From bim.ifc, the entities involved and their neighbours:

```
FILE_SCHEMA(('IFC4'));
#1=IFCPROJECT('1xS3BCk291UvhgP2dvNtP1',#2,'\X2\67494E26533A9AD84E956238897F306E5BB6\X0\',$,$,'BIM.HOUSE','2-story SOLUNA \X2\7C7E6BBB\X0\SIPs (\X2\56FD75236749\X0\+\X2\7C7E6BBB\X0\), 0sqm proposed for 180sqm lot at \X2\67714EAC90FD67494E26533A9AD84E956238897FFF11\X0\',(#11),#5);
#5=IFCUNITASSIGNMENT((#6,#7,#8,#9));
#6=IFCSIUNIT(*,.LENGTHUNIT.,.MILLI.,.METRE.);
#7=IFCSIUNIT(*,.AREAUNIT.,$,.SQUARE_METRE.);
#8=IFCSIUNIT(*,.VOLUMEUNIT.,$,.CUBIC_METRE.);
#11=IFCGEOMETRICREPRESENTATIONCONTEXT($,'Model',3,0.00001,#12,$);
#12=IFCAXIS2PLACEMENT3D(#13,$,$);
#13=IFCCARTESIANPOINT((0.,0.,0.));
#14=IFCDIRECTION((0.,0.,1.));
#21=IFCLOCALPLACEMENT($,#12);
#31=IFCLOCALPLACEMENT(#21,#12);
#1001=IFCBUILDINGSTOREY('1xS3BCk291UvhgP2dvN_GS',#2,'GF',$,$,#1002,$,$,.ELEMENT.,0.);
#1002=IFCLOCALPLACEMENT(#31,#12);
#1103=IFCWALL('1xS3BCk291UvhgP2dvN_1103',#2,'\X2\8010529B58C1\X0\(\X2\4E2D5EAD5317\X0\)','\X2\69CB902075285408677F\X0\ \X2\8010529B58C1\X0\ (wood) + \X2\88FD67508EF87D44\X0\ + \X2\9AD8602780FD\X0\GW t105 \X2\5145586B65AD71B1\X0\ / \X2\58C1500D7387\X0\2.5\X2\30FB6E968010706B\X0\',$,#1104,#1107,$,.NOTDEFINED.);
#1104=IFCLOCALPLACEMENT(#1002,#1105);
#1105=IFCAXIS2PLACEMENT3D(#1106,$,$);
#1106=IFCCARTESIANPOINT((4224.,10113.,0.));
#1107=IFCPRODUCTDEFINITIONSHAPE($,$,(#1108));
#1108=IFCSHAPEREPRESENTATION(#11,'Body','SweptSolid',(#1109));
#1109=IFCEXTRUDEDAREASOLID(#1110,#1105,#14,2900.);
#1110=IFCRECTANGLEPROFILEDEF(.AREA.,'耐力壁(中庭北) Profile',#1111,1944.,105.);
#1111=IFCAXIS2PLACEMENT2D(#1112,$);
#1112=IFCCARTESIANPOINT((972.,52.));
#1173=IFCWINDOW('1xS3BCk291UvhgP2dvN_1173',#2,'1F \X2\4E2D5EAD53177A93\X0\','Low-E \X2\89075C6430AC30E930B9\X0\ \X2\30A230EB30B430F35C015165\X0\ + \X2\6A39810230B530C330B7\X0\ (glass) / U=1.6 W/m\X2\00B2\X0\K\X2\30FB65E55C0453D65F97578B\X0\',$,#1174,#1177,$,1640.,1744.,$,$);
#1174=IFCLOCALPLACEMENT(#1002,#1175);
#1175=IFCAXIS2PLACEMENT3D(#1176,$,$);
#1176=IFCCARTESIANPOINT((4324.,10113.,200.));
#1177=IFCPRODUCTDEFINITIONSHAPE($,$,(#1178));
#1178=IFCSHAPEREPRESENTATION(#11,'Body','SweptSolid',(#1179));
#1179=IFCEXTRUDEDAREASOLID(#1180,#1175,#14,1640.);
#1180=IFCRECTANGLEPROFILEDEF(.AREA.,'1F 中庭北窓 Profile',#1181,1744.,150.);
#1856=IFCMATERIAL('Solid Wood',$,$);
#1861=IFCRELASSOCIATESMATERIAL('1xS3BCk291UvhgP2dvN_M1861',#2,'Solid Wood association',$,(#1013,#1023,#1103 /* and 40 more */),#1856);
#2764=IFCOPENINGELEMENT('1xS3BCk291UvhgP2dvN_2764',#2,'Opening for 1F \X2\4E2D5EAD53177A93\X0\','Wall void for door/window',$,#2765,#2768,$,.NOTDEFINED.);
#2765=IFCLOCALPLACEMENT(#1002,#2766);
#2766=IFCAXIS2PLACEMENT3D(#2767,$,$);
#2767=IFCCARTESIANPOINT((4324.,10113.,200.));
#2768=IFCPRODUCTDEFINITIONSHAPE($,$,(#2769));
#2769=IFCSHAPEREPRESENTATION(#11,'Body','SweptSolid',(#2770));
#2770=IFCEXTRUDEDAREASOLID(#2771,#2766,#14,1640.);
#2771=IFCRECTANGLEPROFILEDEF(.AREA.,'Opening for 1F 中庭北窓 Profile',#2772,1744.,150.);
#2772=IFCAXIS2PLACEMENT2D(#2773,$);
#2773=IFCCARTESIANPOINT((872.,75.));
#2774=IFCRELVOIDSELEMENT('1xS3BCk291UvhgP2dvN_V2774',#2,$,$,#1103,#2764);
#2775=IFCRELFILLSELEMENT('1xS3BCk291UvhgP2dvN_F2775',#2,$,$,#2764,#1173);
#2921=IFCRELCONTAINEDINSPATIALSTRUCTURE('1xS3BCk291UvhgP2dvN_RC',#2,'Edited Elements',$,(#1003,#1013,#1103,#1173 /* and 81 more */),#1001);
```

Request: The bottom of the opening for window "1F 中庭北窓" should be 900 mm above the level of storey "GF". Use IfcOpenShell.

```python
import numpy as np
import ifcopenshell
import ifcopenshell.api.geometry
import ifcopenshell.geom
import ifcopenshell.util.element
import ifcopenshell.util.placement
import ifcopenshell.util.shape
import ifcopenshell.util.unit

model = ifcopenshell.open("bim.ifc")
unit_scale = ifcopenshell.util.unit.calculate_unit_scale(model)

window = model.by_id(1173)
opening = window.FillsVoids[0].RelatingOpeningElement
storey = ifcopenshell.util.element.get_container(window, ifc_class="IfcBuildingStorey")
level = ifcopenshell.util.placement.get_local_placement(storey.ObjectPlacement)[2, 3]

# The opening's origin need not be at the sill, so measure its lowest point.
shape = ifcopenshell.geom.create_shape(ifcopenshell.geom.settings(), opening)
bottom = ifcopenshell.util.shape.get_shape_bottom_elevation(shape, shape.geometry) / unit_scale
dz = level + 0.9 / unit_scale - bottom

shift = np.array([0.0, 0.0, dz])
# The window is not placed relative to its opening, so move both.
for product in (opening, window):
    matrix = ifcopenshell.util.placement.get_local_placement(product.ObjectPlacement)
    matrix[:3, 3] += shift
    ifcopenshell.api.geometry.edit_object_placement(model, product=product, matrix=matrix, is_si=False)

print(f"moved by {dz * unit_scale:+.3f} m")

model.write("bim-out.ifc")
```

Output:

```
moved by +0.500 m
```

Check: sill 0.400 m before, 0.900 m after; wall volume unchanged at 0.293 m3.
